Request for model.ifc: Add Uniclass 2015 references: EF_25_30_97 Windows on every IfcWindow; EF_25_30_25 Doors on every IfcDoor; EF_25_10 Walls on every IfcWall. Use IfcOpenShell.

First a look at what the model holds.

```python
import ifcopenshell

model = ifcopenshell.open("model.ifc")
print(model.schema)
print("classifications:", [c.Name for c in model.by_type("IfcClassification")])
for ifc_class in ("IfcDoor", "IfcRoof", "IfcStair", "IfcWall", "IfcWindow"):
    print(ifc_class, len(model.by_type(ifc_class)))
```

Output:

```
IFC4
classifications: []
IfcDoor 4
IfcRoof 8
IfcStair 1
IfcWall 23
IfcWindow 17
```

```python
import ifcopenshell
import ifcopenshell.api.classification

model = ifcopenshell.open("model.ifc")

system = ifcopenshell.api.classification.add_classification(model, classification="Uniclass 2015")

codes = {
    "IfcWindow": ("EF_25_30_97", "Windows"),
    "IfcDoor": ("EF_25_30_25", "Doors"),
    "IfcWall": ("EF_25_10", "Walls"),
}
for ifc_class, (code, name) in codes.items():
    products = model.by_type(ifc_class)
    ifcopenshell.api.classification.add_reference(
        model, products=products, classification=system, identification=code, name=name
    )
    print(code, len(products))

model.write("model-out.ifc")
```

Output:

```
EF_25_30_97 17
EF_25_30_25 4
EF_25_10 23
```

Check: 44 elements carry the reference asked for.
